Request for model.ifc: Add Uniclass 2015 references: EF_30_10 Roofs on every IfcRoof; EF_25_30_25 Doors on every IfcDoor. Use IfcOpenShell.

First a look at what the model holds.

```python
import ifcopenshell

model = ifcopenshell.open("model.ifc")
print(model.schema)
print("classifications:", [c.Name for c in model.by_type("IfcClassification")])
for ifc_class in ("IfcDoor", "IfcRoof", "IfcStair", "IfcWall", "IfcWindow"):
    print(ifc_class, len(model.by_type(ifc_class)))
```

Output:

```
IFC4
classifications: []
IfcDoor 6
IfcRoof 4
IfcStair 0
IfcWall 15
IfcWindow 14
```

```python
import ifcopenshell
import ifcopenshell.api.classification

model = ifcopenshell.open("model.ifc")

system = ifcopenshell.api.classification.add_classification(model, classification="Uniclass 2015")

codes = {
    "IfcRoof": ("EF_30_10", "Roofs"),
    "IfcDoor": ("EF_25_30_25", "Doors"),
}
for ifc_class, (code, name) in codes.items():
    products = model.by_type(ifc_class)
    ifcopenshell.api.classification.add_reference(
        model, products=products, classification=system, identification=code, name=name
    )
    print(code, len(products))

model.write("model_updated.ifc")
```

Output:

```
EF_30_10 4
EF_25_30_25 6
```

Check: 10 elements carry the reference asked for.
